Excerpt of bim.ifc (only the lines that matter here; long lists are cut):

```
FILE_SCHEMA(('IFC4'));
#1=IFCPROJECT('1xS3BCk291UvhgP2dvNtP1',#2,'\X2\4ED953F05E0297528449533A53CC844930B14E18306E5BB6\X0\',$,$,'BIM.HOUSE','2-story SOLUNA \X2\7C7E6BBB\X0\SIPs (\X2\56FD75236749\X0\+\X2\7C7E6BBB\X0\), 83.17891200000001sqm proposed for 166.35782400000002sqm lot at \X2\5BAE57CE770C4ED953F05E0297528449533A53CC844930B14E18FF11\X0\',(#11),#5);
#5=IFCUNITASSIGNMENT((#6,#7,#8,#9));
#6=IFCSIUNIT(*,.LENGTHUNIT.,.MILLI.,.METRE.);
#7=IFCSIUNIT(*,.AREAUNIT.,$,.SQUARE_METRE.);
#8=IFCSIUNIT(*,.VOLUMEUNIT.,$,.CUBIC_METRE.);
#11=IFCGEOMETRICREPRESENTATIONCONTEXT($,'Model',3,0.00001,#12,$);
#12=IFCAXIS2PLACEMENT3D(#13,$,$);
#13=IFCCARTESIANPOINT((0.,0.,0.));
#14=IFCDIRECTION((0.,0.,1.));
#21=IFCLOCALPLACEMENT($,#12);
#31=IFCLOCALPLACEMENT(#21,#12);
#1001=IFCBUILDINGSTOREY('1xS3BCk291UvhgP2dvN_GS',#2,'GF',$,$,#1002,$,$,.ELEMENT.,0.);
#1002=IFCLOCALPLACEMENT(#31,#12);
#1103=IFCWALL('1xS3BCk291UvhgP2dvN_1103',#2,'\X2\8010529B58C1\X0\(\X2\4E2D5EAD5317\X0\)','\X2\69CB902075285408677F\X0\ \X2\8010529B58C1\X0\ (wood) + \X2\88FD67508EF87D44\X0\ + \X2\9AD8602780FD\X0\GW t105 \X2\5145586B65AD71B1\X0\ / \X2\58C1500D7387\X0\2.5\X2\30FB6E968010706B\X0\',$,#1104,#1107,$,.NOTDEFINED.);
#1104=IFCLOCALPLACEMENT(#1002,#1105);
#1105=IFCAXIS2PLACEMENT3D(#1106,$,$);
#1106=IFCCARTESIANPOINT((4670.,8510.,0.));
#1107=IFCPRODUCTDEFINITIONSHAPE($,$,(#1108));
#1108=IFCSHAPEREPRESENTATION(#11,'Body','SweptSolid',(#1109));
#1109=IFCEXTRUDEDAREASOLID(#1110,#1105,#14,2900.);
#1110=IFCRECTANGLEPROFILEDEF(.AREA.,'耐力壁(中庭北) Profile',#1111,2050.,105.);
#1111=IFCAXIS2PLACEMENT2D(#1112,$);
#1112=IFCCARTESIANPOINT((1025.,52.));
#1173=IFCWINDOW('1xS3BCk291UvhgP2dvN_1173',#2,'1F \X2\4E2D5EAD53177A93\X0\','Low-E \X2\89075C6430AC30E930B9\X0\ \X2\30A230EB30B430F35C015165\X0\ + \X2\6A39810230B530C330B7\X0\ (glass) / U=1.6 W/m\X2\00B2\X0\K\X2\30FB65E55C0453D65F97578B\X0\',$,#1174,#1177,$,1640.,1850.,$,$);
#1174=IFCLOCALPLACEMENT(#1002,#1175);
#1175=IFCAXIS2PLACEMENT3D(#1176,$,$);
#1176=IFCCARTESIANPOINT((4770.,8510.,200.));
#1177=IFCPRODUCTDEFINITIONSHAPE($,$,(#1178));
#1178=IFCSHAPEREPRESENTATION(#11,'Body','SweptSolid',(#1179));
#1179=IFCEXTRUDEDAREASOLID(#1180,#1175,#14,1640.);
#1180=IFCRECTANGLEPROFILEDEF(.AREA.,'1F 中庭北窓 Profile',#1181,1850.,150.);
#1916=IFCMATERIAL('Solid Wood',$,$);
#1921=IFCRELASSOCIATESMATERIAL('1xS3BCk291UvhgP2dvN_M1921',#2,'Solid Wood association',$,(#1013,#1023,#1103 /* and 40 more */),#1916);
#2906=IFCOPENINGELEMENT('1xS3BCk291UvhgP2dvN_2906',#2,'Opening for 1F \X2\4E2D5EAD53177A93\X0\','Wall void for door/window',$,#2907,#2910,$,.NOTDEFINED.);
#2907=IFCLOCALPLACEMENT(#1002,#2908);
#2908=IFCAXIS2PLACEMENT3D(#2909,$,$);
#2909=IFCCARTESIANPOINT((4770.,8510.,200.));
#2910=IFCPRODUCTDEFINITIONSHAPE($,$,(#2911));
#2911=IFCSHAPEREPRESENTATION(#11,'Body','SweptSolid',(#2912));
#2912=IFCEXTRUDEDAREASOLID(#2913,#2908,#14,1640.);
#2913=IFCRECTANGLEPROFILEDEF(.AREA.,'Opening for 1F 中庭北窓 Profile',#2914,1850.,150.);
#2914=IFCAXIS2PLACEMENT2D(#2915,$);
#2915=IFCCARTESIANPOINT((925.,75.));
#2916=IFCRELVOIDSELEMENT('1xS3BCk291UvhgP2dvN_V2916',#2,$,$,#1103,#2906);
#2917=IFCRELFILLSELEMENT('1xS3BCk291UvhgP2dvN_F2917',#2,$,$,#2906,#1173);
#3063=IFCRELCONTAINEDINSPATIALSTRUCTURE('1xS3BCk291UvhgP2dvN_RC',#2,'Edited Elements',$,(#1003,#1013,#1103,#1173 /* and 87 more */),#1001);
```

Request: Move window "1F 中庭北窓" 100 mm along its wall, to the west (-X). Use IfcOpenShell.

```python
import ifcopenshell
import ifcopenshell.api.geometry
import ifcopenshell.util.placement
import ifcopenshell.util.unit

model = ifcopenshell.open("bim.ifc")
unit_scale = ifcopenshell.util.unit.calculate_unit_scale(model)

window = model.by_guid("1xS3BCk291UvhgP2dvN_1173")
opening = window.FillsVoids[0].RelatingOpeningElement
wall = opening.VoidsElements[0].RelatingBuildingElement

wall_matrix = ifcopenshell.util.placement.get_local_placement(wall.ObjectPlacement)
shift = wall_matrix[:3, 0] * -0.1 / unit_scale
before = ifcopenshell.util.placement.get_local_placement(window.ObjectPlacement)[:3, 3].copy()

# The window is not placed relative to its opening, so move both.
for product in (opening, window):
    matrix = ifcopenshell.util.placement.get_local_placement(product.ObjectPlacement)
    matrix[:3, 3] += shift
    ifcopenshell.api.geometry.edit_object_placement(model, product=product, matrix=matrix, is_si=False)

after = ifcopenshell.util.placement.get_local_placement(window.ObjectPlacement)[:3, 3]
print("window moved by", (after - before).round(3) + 0.0)

model.write("bim_edited.ifc")
```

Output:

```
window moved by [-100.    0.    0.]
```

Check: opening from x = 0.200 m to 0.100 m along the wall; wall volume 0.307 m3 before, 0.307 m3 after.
